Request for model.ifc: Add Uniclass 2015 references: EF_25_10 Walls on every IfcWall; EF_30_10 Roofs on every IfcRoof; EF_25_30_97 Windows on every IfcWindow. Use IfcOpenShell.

First a look at what the model holds.

```python
import ifcopenshell

model = ifcopenshell.open("model.ifc")
print(model.schema)
print("classifications:", [c.Name for c in model.by_type("IfcClassification")])
for ifc_class in ("IfcDoor", "IfcRoof", "IfcStair", "IfcWall", "IfcWindow"):
    print(ifc_class, len(model.by_type(ifc_class)))
```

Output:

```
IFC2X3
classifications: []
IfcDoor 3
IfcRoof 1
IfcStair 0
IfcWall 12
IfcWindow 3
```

```python
import ifcopenshell
import ifcopenshell.api.classification

model = ifcopenshell.open("model.ifc")

# IFC2X3 requires Source and Edition and has no link from the project to the system.
system = model.create_entity("IfcClassification", Source="NBS", Edition="2015", Name="Uniclass 2015")

codes = {
    "IfcWall": ("EF_25_10", "Walls"),
    "IfcRoof": ("EF_30_10", "Roofs"),
    "IfcWindow": ("EF_25_30_97", "Windows"),
}
for ifc_class, (code, name) in codes.items():
    products = model.by_type(ifc_class)
    ifcopenshell.api.classification.add_reference(
        model, products=products, classification=system, identification=code, name=name
    )
    print(code, len(products))

model.write("model_updated.ifc")
```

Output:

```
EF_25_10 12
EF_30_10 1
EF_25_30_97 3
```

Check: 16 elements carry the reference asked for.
